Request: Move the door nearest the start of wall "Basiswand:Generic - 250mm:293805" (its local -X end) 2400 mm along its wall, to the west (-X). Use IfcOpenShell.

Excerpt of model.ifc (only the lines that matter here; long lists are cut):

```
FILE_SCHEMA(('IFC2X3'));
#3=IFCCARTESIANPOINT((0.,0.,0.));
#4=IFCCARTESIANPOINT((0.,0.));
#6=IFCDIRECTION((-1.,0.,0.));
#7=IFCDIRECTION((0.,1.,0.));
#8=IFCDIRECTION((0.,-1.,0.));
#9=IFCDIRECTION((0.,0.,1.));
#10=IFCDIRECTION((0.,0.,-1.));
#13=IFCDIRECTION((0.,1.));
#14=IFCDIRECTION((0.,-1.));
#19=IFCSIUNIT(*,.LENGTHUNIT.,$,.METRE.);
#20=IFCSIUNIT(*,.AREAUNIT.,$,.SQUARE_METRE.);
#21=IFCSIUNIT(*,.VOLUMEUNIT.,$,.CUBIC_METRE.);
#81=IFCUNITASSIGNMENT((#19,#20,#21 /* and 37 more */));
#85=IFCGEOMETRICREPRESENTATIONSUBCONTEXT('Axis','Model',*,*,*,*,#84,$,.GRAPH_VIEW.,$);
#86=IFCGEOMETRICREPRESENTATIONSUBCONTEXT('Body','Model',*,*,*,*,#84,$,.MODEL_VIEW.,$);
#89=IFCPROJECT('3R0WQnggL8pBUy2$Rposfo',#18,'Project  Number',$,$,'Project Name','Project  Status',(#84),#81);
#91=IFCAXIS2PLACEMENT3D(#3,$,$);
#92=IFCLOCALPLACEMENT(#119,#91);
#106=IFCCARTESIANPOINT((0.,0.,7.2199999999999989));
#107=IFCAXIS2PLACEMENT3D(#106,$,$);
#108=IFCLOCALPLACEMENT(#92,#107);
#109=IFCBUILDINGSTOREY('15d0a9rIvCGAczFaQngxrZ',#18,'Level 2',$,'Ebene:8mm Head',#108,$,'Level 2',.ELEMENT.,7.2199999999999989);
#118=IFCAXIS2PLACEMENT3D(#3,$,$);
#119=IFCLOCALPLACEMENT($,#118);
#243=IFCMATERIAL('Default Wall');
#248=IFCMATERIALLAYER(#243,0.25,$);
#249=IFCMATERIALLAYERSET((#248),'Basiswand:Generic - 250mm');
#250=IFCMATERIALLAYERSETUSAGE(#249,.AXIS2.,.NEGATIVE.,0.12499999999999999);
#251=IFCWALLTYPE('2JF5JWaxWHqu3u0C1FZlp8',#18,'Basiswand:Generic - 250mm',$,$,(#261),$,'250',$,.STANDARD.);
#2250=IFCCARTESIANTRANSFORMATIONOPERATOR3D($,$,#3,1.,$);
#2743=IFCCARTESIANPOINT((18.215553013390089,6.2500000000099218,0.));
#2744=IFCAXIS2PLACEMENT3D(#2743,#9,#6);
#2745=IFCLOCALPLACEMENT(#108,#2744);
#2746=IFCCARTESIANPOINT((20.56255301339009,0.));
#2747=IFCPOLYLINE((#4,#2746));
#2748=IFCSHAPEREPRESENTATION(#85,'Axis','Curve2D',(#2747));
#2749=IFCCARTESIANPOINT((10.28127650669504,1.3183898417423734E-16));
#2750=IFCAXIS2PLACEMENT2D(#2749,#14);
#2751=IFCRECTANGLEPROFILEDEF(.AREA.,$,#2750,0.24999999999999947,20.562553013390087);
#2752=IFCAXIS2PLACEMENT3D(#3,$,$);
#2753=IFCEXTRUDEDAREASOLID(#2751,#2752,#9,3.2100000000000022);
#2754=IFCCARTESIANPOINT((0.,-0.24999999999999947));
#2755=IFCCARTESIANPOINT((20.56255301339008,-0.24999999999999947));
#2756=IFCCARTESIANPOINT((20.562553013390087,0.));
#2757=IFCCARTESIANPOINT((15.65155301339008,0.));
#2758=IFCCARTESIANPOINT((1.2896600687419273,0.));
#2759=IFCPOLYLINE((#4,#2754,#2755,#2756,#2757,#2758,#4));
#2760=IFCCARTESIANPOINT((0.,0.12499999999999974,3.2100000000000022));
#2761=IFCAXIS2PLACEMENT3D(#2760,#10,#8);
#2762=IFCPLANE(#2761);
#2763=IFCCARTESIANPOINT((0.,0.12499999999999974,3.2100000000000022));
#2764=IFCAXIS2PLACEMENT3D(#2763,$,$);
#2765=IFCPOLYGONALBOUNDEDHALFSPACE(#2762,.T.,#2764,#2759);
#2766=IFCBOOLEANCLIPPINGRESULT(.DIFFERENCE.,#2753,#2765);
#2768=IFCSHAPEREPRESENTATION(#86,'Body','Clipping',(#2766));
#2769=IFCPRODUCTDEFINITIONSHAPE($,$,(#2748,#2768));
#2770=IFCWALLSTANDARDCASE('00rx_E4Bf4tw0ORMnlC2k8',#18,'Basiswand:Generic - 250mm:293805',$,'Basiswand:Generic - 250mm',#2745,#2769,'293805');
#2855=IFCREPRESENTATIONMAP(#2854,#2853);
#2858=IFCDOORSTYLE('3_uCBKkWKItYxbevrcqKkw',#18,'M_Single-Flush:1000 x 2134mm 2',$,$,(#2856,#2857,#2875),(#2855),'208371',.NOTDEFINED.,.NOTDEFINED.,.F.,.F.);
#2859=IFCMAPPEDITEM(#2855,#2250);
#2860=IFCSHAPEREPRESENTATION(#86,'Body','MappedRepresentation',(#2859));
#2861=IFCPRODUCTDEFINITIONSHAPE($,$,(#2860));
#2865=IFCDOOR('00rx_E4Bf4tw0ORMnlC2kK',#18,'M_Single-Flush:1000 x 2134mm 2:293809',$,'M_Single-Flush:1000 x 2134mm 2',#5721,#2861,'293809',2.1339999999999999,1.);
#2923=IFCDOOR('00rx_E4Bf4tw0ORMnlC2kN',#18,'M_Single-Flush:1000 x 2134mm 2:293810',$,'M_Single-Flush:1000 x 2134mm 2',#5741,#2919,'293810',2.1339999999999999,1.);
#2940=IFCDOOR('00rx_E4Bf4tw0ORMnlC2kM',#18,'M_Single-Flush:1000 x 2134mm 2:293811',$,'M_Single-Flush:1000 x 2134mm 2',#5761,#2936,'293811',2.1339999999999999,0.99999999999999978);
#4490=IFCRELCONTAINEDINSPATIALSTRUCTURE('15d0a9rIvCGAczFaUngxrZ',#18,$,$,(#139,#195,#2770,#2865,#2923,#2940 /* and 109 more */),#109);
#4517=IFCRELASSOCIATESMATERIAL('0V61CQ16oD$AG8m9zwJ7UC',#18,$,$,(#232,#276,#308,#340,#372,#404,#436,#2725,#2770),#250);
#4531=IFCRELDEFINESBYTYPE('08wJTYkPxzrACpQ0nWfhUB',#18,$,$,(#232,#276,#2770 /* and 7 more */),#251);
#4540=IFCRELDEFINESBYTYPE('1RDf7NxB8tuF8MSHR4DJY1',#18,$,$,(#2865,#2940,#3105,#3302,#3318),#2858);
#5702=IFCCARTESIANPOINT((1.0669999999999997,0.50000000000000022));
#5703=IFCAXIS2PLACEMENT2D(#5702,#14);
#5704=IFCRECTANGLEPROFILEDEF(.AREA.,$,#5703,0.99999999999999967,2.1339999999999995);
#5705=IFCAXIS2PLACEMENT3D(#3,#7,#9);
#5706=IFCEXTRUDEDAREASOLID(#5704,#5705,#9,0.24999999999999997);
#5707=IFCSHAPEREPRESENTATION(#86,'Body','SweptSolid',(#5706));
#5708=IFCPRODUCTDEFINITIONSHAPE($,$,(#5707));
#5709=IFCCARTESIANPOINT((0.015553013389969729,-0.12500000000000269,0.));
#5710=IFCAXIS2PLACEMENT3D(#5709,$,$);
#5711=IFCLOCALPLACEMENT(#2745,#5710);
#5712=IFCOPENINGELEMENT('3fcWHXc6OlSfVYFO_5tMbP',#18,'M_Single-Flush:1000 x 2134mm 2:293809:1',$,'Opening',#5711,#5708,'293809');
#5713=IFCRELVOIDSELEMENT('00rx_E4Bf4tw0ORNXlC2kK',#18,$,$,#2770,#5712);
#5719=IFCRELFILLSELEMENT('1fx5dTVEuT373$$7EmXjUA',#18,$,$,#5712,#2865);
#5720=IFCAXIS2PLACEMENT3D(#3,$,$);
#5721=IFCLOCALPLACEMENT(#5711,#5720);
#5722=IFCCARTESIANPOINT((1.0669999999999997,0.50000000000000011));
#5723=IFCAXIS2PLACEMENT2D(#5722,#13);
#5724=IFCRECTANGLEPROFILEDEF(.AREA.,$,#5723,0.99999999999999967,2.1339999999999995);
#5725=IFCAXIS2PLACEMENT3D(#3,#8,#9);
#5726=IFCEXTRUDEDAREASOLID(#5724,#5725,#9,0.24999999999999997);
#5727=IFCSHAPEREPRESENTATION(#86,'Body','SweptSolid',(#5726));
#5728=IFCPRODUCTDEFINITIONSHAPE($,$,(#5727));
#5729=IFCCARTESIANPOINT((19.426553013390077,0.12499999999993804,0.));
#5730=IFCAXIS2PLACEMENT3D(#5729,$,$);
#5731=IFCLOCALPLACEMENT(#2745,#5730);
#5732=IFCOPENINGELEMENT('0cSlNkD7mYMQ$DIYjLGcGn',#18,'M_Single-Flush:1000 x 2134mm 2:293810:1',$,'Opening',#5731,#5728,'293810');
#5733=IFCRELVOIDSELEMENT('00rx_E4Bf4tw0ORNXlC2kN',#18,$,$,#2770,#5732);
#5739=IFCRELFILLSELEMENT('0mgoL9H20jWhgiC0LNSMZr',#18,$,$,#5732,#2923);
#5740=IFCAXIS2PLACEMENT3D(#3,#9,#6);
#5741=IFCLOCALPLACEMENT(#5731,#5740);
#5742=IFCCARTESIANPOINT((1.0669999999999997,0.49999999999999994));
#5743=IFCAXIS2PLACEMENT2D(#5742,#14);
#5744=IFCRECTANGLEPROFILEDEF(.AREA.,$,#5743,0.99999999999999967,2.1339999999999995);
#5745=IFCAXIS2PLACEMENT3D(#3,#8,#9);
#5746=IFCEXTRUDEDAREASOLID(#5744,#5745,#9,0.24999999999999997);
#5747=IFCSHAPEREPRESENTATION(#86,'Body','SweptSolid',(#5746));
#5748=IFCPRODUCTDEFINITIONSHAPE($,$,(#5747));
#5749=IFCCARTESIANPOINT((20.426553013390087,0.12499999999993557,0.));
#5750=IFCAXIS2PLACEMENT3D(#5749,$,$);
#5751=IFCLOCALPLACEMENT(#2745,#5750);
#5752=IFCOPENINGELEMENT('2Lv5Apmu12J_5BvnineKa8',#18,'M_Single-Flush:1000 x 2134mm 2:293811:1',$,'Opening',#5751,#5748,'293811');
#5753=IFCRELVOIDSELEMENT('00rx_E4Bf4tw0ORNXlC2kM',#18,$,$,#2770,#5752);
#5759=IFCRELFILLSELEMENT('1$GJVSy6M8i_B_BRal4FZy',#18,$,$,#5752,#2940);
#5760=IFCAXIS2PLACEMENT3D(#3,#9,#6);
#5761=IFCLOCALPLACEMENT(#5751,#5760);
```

```python
import ifcopenshell
import ifcopenshell.api.geometry
import ifcopenshell.util.placement
import ifcopenshell.util.unit

model = ifcopenshell.open("model.ifc")
unit_scale = ifcopenshell.util.unit.calculate_unit_scale(model)

door = model.by_id(2865)
opening = door.FillsVoids[0].RelatingOpeningElement
wall = opening.VoidsElements[0].RelatingBuildingElement

wall_matrix = ifcopenshell.util.placement.get_local_placement(wall.ObjectPlacement)
shift = wall_matrix[:3, 0] * 2.4 / unit_scale
before = ifcopenshell.util.placement.get_local_placement(door.ObjectPlacement)[:3, 3].copy()

# The door is placed relative to its opening, so it follows when the opening moves.
matrix = ifcopenshell.util.placement.get_local_placement(opening.ObjectPlacement)
matrix[:3, 3] += shift
ifcopenshell.api.geometry.edit_object_placement(
    model, product=opening, matrix=matrix, is_si=False, should_transform_children=True
)

after = ifcopenshell.util.placement.get_local_placement(door.ObjectPlacement)[:3, 3]
print("door moved by", (after - before).round(3) + 0.0)

model.write("model-out.ifc")
```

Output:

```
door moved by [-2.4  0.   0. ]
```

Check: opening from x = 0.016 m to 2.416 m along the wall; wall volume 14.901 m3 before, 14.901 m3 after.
